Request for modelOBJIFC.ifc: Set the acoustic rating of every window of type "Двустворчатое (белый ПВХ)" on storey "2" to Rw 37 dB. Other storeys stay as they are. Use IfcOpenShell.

First a look at what the model holds.

```python
import ifcopenshell
import ifcopenshell.util.element

model = ifcopenshell.open("modelOBJIFC.ifc")
print(model.schema)
storey = next(s for s in model.by_type("IfcBuildingStorey") if s.Name == "2")
windows = [e for e in ifcopenshell.util.element.get_decomposition(storey) if e.is_a("IfcWindow")]
seen = {}
for e in windows:
    element_type = ifcopenshell.util.element.get_type(e)
    key = (element_type.Name if element_type != e and element_type else None, ifcopenshell.util.element.get_pset(e, "Pset_WindowCommon", "AcousticRating"))
    seen[key] = seen.get(key, 0) + 1
for (name, value), count in sorted(seen.items(), key=str):
    print(count, "x", name, "|", value)
```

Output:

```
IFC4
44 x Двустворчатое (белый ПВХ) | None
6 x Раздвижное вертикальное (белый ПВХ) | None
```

```python
import ifcopenshell
import ifcopenshell.api.pset
import ifcopenshell.util.element

model = ifcopenshell.open("modelOBJIFC.ifc")

storey = next(s for s in model.by_type("IfcBuildingStorey") if s.Name == "2")
windows = [e for e in ifcopenshell.util.element.get_decomposition(storey) if e.is_a("IfcWindow")]

count = 0
for e in windows:
    element_type = ifcopenshell.util.element.get_type(e)
    if element_type in (None, e) or element_type.Name != "Двустворчатое (белый ПВХ)":
        continue
    # add_pset returns the element's existing set when there is one.
    pset = ifcopenshell.api.pset.add_pset(model, product=e, name="Pset_WindowCommon")
    ifcopenshell.api.pset.edit_pset(model, pset=pset, properties={"AcousticRating": "Rw 37 dB"})
    count += 1

print(count, "windows updated")

model.write("modelOBJIFC_rev.ifc")
```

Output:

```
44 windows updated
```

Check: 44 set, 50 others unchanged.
